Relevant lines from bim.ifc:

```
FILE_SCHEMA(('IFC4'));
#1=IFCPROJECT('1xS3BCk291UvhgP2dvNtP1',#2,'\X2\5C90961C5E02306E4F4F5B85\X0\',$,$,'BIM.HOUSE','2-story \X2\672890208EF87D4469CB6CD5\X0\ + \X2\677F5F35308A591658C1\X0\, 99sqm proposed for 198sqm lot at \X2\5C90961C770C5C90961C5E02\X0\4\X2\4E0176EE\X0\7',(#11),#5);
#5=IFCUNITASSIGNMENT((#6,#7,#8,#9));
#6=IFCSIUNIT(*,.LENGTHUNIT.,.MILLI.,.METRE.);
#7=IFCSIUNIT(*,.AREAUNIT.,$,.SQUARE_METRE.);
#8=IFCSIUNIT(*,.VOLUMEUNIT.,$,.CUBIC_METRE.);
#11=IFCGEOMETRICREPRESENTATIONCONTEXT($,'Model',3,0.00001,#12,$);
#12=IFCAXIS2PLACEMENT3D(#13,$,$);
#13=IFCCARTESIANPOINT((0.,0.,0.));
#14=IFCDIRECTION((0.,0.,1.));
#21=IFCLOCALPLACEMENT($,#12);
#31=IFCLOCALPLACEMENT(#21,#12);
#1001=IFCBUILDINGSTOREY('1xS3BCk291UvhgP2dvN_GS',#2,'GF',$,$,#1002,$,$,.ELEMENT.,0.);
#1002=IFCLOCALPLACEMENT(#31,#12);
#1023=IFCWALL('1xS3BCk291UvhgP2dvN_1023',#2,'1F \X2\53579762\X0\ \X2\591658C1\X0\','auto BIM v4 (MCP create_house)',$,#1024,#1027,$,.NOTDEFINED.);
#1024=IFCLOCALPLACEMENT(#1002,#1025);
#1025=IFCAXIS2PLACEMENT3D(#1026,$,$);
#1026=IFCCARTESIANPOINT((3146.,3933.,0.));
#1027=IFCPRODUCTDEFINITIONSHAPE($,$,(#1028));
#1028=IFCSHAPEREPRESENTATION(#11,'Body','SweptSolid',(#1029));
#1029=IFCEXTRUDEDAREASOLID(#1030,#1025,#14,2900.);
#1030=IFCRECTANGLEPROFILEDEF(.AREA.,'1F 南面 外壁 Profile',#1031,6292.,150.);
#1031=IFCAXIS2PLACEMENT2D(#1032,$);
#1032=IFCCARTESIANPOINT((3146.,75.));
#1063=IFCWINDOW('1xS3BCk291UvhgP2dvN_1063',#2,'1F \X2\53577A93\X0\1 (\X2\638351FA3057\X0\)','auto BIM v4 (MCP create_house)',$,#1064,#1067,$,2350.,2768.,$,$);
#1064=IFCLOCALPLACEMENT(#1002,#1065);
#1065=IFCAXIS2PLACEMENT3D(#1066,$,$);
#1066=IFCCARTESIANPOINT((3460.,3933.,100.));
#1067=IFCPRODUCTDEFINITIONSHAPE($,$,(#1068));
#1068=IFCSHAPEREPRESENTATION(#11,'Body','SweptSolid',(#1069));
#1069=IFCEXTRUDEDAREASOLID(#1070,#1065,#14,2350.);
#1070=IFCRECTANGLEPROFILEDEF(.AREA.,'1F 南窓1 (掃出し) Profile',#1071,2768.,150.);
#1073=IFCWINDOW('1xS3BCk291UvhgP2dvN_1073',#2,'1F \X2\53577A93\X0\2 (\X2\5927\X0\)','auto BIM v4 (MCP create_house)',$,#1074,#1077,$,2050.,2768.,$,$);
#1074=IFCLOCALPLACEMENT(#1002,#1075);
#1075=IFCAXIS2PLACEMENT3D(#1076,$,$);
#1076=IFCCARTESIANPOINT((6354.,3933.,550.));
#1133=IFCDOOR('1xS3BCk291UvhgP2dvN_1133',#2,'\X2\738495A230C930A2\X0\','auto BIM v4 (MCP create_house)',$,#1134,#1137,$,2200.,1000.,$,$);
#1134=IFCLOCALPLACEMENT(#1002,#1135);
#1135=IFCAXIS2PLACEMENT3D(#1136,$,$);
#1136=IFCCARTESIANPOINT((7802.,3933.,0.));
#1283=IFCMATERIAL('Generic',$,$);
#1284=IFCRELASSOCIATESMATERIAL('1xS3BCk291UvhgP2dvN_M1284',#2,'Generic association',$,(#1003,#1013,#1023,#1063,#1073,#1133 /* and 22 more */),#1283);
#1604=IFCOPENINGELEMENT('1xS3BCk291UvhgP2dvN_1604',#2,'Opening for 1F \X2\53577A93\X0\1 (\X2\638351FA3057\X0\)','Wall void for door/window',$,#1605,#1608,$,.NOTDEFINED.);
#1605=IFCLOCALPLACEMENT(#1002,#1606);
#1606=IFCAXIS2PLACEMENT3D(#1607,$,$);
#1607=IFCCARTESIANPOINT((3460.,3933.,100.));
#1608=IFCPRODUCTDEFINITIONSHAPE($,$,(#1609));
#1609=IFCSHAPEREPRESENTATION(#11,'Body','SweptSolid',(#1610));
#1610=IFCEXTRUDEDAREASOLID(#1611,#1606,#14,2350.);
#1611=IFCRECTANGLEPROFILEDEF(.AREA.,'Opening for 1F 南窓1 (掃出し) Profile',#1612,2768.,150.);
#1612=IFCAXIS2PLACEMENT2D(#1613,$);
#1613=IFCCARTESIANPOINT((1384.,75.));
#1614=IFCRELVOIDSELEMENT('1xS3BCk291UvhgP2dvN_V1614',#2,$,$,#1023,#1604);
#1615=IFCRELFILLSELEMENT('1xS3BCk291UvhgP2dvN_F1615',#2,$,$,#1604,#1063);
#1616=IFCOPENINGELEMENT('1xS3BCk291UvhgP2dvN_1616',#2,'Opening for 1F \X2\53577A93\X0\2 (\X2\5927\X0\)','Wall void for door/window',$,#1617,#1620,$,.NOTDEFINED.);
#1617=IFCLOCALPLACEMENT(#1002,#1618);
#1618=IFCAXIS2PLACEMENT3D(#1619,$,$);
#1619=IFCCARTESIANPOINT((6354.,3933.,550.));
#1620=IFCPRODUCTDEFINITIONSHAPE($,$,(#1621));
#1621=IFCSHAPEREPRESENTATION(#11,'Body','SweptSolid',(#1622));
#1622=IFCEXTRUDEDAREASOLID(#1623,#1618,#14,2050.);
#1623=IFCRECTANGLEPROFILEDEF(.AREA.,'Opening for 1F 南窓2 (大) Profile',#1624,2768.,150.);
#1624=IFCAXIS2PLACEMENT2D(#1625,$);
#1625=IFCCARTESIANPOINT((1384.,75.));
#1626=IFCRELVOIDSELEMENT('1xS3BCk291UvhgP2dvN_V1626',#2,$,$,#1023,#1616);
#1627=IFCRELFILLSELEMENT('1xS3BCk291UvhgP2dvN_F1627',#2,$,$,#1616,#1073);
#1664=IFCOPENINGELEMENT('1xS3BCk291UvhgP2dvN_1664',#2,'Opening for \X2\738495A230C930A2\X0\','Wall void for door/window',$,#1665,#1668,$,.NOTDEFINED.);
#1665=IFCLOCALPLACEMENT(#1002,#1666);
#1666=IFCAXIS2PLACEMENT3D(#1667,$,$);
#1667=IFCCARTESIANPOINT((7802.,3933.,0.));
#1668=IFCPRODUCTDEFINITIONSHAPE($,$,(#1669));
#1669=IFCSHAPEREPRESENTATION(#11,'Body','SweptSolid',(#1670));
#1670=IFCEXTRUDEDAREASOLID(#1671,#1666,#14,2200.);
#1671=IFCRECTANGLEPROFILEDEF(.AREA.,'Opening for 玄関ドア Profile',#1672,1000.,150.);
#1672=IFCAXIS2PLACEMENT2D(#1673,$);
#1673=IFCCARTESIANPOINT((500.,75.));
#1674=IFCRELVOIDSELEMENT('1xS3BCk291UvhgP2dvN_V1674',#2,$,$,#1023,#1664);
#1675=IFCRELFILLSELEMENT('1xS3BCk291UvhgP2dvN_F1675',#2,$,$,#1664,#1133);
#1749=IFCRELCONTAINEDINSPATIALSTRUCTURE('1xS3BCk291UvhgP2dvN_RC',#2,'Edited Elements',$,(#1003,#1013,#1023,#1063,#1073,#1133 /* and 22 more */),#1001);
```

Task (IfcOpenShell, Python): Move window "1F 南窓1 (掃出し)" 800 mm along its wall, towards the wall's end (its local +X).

```python
import ifcopenshell
import ifcopenshell.api.geometry
import ifcopenshell.util.placement
import ifcopenshell.util.unit

model = ifcopenshell.open("bim.ifc")
unit_scale = ifcopenshell.util.unit.calculate_unit_scale(model)

window = model.by_guid("1xS3BCk291UvhgP2dvN_1063")
opening = window.FillsVoids[0].RelatingOpeningElement
wall = opening.VoidsElements[0].RelatingBuildingElement

wall_matrix = ifcopenshell.util.placement.get_local_placement(wall.ObjectPlacement)
shift = wall_matrix[:3, 0] * 0.8 / unit_scale
before = ifcopenshell.util.placement.get_local_placement(window.ObjectPlacement)[:3, 3].copy()

# The window is not placed relative to its opening, so move both.
for product in (opening, window):
    matrix = ifcopenshell.util.placement.get_local_placement(product.ObjectPlacement)
    matrix[:3, 3] += shift
    ifcopenshell.api.geometry.edit_object_placement(model, product=product, matrix=matrix, is_si=False)

after = ifcopenshell.util.placement.get_local_placement(window.ObjectPlacement)[:3, 3]
print("window moved by", (after - before).round(3) + 0.0)

model.write("bim_v2.ifc")
```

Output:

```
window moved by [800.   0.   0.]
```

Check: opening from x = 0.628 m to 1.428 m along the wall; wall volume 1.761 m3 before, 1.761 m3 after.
